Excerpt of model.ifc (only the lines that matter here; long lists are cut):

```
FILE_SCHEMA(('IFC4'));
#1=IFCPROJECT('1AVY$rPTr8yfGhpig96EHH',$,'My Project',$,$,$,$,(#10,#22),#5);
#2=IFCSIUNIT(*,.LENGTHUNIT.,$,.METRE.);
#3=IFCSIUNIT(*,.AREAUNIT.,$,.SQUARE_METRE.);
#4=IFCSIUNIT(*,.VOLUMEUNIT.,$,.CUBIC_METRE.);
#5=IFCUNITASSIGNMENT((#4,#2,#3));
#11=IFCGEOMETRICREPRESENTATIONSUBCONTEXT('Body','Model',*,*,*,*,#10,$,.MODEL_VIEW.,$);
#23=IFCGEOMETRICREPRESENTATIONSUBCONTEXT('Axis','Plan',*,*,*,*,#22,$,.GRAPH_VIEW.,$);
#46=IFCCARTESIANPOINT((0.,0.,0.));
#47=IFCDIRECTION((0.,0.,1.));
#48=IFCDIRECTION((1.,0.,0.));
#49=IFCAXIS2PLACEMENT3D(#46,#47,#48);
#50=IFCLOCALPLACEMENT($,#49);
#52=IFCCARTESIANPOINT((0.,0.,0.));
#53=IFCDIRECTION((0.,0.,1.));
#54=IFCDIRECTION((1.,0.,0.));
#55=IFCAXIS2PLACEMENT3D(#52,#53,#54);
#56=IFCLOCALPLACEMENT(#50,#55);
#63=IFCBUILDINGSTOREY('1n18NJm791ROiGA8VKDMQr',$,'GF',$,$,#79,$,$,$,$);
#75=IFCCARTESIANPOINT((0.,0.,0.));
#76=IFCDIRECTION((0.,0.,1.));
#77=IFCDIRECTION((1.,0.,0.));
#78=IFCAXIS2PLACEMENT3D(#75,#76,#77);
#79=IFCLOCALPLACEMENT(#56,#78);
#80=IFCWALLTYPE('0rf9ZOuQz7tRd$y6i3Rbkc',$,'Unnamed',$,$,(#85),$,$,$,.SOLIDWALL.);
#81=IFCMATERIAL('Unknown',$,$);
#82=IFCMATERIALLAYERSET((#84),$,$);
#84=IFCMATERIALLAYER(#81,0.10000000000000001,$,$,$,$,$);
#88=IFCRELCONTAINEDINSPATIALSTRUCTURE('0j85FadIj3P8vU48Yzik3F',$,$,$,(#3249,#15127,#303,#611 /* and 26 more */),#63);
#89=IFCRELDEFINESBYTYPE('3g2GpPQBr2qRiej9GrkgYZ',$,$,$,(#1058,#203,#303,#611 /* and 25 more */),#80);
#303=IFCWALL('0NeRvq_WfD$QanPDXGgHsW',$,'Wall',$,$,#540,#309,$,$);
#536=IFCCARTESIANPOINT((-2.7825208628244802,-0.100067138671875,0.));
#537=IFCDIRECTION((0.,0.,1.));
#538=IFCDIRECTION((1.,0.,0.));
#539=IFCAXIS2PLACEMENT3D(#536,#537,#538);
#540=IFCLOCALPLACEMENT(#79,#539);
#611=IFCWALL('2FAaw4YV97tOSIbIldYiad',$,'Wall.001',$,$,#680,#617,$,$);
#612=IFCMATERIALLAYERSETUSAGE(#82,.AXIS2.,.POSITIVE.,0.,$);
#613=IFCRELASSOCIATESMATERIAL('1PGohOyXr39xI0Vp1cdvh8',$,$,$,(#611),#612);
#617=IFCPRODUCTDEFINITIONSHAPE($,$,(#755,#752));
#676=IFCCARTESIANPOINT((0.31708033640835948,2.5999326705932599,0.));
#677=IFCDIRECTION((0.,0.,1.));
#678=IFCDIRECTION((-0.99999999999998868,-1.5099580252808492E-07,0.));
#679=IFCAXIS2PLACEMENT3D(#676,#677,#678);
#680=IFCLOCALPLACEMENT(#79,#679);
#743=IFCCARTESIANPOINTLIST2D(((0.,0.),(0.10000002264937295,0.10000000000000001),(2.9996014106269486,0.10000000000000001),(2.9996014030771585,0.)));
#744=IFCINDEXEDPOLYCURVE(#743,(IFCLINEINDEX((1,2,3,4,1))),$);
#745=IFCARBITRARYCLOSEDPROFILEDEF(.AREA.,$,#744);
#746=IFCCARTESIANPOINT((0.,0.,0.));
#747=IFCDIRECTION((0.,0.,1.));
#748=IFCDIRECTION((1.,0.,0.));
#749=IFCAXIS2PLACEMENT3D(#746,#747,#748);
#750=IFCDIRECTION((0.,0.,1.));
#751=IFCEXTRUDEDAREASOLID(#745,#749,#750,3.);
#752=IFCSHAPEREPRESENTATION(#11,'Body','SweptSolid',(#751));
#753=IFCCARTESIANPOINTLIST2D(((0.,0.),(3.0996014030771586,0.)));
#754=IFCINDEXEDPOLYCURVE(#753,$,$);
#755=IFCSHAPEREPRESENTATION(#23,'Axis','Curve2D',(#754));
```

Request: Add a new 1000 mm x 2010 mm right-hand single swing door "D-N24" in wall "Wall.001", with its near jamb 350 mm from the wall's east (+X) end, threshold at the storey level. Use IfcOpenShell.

```python
import numpy as np
import ifcopenshell
import ifcopenshell.api.feature
import ifcopenshell.api.geometry
import ifcopenshell.api.root
import ifcopenshell.api.spatial
import ifcopenshell.geom
import ifcopenshell.util.element
import ifcopenshell.util.placement
import ifcopenshell.util.representation
import ifcopenshell.util.shape
import ifcopenshell.util.unit

model = ifcopenshell.open("model.ifc")
unit_scale = ifcopenshell.util.unit.calculate_unit_scale(model)
settings = ifcopenshell.geom.settings()


def volume(element):
    """Net volume in cubic metres, openings subtracted."""
    shape = ifcopenshell.geom.create_shape(settings, element)
    return ifcopenshell.util.shape.get_volume(shape.geometry)


wall = model.by_guid("2FAaw4YV97tOSIbIldYiad")
storey = ifcopenshell.util.element.get_container(wall, ifc_class="IfcBuildingStorey")
context = ifcopenshell.util.representation.get_context(model, "Model", "Body", "MODEL_VIEW")
before = volume(wall)

width, height, from_end, sill = 1, 2.01, 0.35, 0.0  # metres

# The wall runs along its own X axis, and the end named is its -X end.
wall_shape = ifcopenshell.geom.create_shape(settings, wall)
x, y, z = ifcopenshell.util.shape.get_vertices(wall_shape.geometry).T
start = x.min() + from_end
face, thickness = float(y.min()), float(y.max() - y.min())
wall_matrix = ifcopenshell.util.placement.get_local_placement(wall.ObjectPlacement)
level = ifcopenshell.util.placement.get_local_placement(storey.ObjectPlacement)[2, 3]


def in_wall(x, y):
    """Placement at x, y metres in the wall's axes, at sill height."""
    matrix = wall_matrix.copy()
    matrix[:, 3] = wall_matrix @ np.array([x / unit_scale, y / unit_scale, 0.0, 1.0])
    matrix[2, 3] = level + sill / unit_scale
    return matrix


# Opening: a box that overshoots both wall faces by 50 mm.
opening = ifcopenshell.api.root.create_entity(model, ifc_class="IfcOpeningElement", predefined_type="OPENING")
box = ifcopenshell.api.geometry.add_wall_representation(
    model, context=context, length=width, height=height, thickness=thickness + 0.1
)
ifcopenshell.api.geometry.assign_representation(model, product=opening, representation=box)
ifcopenshell.api.geometry.edit_object_placement(model, product=opening, matrix=in_wall(start, face - 0.05), is_si=False)
ifcopenshell.api.feature.add_feature(model, feature=opening, element=wall)

door = ifcopenshell.api.root.create_entity(model, ifc_class="IfcDoor", name="D-N24", predefined_type="DOOR")
door.OverallWidth, door.OverallHeight = width / unit_scale, height / unit_scale
door.OperationType = "SINGLE_SWING_RIGHT"
body = ifcopenshell.api.geometry.add_door_representation(
    model,
    context=context,
    overall_width=door.OverallWidth,
    overall_height=door.OverallHeight,
    operation_type="SINGLE_SWING_RIGHT",
    lining_properties={"LiningDepth": thickness / unit_scale, "ThresholdDepth": thickness / unit_scale},
)
ifcopenshell.api.geometry.assign_representation(model, product=door, representation=body)
ifcopenshell.api.spatial.assign_container(model, products=[door], relating_structure=storey)
ifcopenshell.api.feature.add_filling(model, opening=opening, element=door)

# The lining spans the wall, so the door starts at the wall face.
ifcopenshell.api.geometry.edit_object_placement(model, product=door, matrix=in_wall(start, face), is_si=False)

after = volume(wall)

print(f"wall volume {before:.3f} -> {after:.3f} m3")

model.write("model_edited.ifc")
```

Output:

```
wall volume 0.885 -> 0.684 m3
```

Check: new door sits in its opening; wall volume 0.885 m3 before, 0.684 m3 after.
